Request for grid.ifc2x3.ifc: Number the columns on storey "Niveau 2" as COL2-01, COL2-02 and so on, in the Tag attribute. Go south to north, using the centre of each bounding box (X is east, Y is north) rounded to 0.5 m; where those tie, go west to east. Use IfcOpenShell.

First a look at what the model holds.

```python
import ifcopenshell
import ifcopenshell.util.element
import ifcopenshell.util.placement

model = ifcopenshell.open("grid.ifc2x3.ifc")
print(model.schema)
storey = next(s for s in model.by_type("IfcBuildingStorey") if s.Name == "Niveau 2")
columns = [e for e in ifcopenshell.util.element.get_decomposition(storey) if e.is_a("IfcColumn")]
for e in sorted(columns, key=lambda e: e.id()):
    origin = ifcopenshell.util.placement.get_local_placement(e.ObjectPlacement)[:3, 3]
    print(e.id(), e.Tag, e.Name, origin.round(2) + 0.0, sep=" | ")
```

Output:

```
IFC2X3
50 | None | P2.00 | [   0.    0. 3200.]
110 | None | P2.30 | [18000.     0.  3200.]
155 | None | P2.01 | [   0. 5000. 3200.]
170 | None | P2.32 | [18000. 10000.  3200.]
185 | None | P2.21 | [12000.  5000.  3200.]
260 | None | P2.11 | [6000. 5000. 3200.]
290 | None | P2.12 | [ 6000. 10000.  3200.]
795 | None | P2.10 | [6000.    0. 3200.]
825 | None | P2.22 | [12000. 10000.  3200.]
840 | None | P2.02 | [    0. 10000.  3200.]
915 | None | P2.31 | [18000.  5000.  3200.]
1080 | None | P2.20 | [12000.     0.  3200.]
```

```python
import ifcopenshell
import ifcopenshell.geom
import ifcopenshell.util.element
import ifcopenshell.util.shape

model = ifcopenshell.open("grid.ifc2x3.ifc")
settings = ifcopenshell.geom.settings()
settings.set("use-world-coords", True)


def centre(element):
    shape = ifcopenshell.geom.create_shape(settings, element)
    return ifcopenshell.util.shape.get_bbox_centroid(shape.geometry)


storey = next(s for s in model.by_type("IfcBuildingStorey") if s.Name == "Niveau 2")
columns = [e for e in ifcopenshell.util.element.get_decomposition(storey) if e.is_a("IfcColumn")]

# Insertion points can sit at a corner or the storey origin, so sort by the geometry (in metres).
centres = {e: centre(e) for e in columns}
columns.sort(key=lambda e: (round(centres[e][1] / 0.5), centres[e][0]))

for i, e in enumerate(columns, start=1):
    number = f"COL2-{i:02d}"
    e.Tag = number
    print(e.id(), number)

model.write("grid.ifc2x3-out.ifc")
```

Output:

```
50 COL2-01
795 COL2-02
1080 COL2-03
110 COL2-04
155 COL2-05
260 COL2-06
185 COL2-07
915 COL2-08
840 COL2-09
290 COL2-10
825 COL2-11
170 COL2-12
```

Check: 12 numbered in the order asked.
